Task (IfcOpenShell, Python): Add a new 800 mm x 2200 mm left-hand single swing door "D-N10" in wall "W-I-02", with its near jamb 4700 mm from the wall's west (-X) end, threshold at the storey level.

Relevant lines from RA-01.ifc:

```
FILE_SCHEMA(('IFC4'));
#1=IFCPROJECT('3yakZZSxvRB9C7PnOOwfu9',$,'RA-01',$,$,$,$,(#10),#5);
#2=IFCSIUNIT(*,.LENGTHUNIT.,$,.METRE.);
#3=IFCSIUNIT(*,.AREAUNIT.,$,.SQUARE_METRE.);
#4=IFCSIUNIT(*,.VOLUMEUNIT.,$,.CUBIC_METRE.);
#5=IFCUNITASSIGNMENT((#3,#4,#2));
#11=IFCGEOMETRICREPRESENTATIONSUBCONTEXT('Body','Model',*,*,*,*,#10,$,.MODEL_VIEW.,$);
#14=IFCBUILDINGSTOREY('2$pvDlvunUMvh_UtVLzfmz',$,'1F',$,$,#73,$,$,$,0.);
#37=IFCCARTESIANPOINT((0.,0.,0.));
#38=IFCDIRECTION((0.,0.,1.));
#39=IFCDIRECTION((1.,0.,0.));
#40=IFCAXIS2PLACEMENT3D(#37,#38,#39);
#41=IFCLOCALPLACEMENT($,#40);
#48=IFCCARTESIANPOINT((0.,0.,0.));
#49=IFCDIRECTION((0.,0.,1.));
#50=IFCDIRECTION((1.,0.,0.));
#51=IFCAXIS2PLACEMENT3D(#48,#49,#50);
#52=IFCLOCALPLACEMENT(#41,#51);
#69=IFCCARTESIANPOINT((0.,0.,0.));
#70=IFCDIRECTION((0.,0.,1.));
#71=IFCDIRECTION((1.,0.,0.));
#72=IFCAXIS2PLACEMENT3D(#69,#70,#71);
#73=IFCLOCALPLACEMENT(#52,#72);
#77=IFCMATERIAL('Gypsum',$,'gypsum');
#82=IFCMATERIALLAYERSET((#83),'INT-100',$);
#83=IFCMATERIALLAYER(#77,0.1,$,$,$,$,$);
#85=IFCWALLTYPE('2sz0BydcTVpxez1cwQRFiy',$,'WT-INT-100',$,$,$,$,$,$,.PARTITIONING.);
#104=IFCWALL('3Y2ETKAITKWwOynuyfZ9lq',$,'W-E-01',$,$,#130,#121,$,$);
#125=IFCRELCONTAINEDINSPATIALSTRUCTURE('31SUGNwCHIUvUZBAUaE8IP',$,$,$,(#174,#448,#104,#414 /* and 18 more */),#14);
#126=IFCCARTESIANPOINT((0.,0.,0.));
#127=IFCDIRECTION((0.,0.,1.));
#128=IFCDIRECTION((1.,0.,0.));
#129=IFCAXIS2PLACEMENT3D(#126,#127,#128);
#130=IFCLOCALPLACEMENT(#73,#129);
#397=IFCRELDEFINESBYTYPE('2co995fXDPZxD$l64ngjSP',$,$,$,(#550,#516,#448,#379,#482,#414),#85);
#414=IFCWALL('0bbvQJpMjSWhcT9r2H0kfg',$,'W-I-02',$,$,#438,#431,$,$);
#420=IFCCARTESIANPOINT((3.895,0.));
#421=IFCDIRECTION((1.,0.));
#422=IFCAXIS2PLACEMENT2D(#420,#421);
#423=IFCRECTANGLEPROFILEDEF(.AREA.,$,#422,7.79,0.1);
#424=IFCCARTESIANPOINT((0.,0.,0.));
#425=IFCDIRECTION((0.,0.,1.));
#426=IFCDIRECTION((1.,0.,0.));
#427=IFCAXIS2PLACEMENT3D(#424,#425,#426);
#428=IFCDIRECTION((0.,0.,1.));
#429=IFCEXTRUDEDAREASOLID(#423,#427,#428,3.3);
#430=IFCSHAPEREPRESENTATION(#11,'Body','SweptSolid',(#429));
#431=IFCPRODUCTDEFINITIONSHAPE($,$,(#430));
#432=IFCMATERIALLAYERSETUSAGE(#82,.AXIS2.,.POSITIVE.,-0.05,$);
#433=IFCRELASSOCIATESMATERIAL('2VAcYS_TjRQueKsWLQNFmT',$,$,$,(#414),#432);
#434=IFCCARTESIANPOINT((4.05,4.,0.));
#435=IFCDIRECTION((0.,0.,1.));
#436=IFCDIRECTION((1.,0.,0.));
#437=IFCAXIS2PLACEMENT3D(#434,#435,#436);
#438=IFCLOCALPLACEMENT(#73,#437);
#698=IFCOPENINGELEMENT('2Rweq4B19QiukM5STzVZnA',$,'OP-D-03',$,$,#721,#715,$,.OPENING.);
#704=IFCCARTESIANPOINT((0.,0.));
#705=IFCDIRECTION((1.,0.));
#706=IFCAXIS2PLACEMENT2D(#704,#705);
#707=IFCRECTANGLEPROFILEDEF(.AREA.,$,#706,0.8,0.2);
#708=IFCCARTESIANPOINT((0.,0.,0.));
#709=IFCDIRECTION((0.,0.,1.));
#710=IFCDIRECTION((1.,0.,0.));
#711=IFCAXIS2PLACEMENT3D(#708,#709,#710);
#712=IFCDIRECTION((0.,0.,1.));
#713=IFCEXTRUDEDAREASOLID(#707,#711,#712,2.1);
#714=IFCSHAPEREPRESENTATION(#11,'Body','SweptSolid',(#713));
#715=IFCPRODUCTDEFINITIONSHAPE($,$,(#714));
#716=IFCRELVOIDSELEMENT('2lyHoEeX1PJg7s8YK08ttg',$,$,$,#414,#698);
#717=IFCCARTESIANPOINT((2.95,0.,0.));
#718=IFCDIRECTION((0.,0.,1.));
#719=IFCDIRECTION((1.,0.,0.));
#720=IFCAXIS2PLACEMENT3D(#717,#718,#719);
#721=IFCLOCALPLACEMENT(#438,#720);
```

```python
import numpy as np
import ifcopenshell
import ifcopenshell.api.feature
import ifcopenshell.api.geometry
import ifcopenshell.api.root
import ifcopenshell.api.spatial
import ifcopenshell.geom
import ifcopenshell.util.element
import ifcopenshell.util.placement
import ifcopenshell.util.representation
import ifcopenshell.util.shape
import ifcopenshell.util.unit

model = ifcopenshell.open("RA-01.ifc")
unit_scale = ifcopenshell.util.unit.calculate_unit_scale(model)
settings = ifcopenshell.geom.settings()


def volume(element):
    """Net volume in cubic metres, openings subtracted."""
    shape = ifcopenshell.geom.create_shape(settings, element)
    return ifcopenshell.util.shape.get_volume(shape.geometry)


wall = model.by_guid("0bbvQJpMjSWhcT9r2H0kfg")
storey = ifcopenshell.util.element.get_container(wall, ifc_class="IfcBuildingStorey")
context = ifcopenshell.util.representation.get_context(model, "Model", "Body", "MODEL_VIEW")
before = volume(wall)

width, height, from_end, sill = 0.8, 2.2, 4.7, 0.0  # metres

# The wall runs along its own X axis, and the end named is its -X end.
wall_shape = ifcopenshell.geom.create_shape(settings, wall)
x, y, z = ifcopenshell.util.shape.get_vertices(wall_shape.geometry).T
start = x.min() + from_end
face, thickness = float(y.min()), float(y.max() - y.min())
wall_matrix = ifcopenshell.util.placement.get_local_placement(wall.ObjectPlacement)
level = ifcopenshell.util.placement.get_local_placement(storey.ObjectPlacement)[2, 3]


def in_wall(x, y):
    """Placement at x, y metres in the wall's axes, at sill height."""
    matrix = wall_matrix.copy()
    matrix[:, 3] = wall_matrix @ np.array([x / unit_scale, y / unit_scale, 0.0, 1.0])
    matrix[2, 3] = level + sill / unit_scale
    return matrix


# Opening: a box that overshoots both wall faces by 50 mm.
opening = ifcopenshell.api.root.create_entity(model, ifc_class="IfcOpeningElement", predefined_type="OPENING")
box = ifcopenshell.api.geometry.add_wall_representation(
    model, context=context, length=width, height=height, thickness=thickness + 0.1
)
ifcopenshell.api.geometry.assign_representation(model, product=opening, representation=box)
ifcopenshell.api.geometry.edit_object_placement(model, product=opening, matrix=in_wall(start, face - 0.05), is_si=False)
ifcopenshell.api.feature.add_feature(model, feature=opening, element=wall)

door = ifcopenshell.api.root.create_entity(model, ifc_class="IfcDoor", name="D-N10", predefined_type="DOOR")
door.OverallWidth, door.OverallHeight = width / unit_scale, height / unit_scale
door.OperationType = "SINGLE_SWING_LEFT"
body = ifcopenshell.api.geometry.add_door_representation(
    model,
    context=context,
    overall_width=door.OverallWidth,
    overall_height=door.OverallHeight,
    operation_type="SINGLE_SWING_LEFT",
    lining_properties={"LiningDepth": thickness / unit_scale, "ThresholdDepth": thickness / unit_scale},
)
ifcopenshell.api.geometry.assign_representation(model, product=door, representation=body)
ifcopenshell.api.spatial.assign_container(model, products=[door], relating_structure=storey)
ifcopenshell.api.feature.add_filling(model, opening=opening, element=door)

# The lining spans the wall, so the door starts at the wall face.
ifcopenshell.api.geometry.edit_object_placement(model, product=door, matrix=in_wall(start, face), is_si=False)

after = volume(wall)

print(f"wall volume {before:.3f} -> {after:.3f} m3")

model.write("RA-01_edited.ifc")
```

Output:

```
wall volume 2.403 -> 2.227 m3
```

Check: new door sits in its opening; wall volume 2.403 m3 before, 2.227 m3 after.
